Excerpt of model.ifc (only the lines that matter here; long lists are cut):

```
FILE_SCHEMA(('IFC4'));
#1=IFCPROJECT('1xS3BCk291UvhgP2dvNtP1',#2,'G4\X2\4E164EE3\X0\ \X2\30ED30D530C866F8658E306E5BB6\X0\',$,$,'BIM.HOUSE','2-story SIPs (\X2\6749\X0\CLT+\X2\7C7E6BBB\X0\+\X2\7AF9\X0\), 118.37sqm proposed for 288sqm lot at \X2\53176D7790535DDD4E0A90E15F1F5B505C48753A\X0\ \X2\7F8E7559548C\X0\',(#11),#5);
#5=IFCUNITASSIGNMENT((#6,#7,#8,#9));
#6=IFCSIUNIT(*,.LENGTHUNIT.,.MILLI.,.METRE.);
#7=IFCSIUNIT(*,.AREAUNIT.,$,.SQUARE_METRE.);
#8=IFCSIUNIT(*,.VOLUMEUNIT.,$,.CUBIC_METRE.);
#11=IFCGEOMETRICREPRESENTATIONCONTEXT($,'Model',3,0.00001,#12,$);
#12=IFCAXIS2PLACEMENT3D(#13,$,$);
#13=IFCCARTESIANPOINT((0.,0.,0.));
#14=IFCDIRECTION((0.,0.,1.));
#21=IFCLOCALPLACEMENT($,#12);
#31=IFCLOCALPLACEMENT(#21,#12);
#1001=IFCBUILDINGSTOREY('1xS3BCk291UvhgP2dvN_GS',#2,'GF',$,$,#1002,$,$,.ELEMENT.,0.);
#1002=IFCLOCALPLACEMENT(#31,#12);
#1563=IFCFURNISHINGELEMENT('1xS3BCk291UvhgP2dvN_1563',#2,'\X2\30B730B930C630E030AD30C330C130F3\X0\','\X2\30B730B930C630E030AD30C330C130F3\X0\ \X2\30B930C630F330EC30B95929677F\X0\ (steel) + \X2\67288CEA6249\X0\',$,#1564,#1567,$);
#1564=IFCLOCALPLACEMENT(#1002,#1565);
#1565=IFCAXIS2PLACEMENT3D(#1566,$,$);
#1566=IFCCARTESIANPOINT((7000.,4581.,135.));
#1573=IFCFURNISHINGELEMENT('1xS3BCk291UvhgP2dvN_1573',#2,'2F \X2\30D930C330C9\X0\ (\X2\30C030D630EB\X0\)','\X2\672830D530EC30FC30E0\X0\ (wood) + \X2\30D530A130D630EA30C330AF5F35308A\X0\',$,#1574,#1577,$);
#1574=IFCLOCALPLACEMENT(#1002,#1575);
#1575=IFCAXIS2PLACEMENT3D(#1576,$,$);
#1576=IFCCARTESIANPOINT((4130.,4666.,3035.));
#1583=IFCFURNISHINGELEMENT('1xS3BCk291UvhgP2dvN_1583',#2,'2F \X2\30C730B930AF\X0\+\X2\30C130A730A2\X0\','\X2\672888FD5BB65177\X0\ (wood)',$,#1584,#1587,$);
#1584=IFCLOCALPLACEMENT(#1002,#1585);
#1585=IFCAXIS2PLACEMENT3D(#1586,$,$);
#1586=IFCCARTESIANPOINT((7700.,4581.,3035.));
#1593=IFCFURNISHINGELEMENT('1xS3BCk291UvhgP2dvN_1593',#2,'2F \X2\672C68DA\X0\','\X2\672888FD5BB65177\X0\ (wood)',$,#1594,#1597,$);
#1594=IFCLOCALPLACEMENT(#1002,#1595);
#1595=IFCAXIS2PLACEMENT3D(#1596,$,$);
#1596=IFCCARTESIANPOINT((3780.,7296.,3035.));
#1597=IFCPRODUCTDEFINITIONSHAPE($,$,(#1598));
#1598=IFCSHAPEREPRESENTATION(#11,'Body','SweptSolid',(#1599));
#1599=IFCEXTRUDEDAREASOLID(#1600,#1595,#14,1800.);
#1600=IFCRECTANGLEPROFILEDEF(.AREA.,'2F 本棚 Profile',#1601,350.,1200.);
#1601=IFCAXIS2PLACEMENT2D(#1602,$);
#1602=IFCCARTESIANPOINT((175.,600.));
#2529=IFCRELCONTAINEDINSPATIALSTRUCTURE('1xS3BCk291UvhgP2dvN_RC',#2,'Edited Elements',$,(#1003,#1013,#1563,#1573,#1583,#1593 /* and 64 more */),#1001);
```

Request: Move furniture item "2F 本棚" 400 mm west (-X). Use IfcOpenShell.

```python
import ifcopenshell
import ifcopenshell.api.geometry
import ifcopenshell.util.placement
import ifcopenshell.util.unit

model = ifcopenshell.open("model.ifc")
unit_scale = ifcopenshell.util.unit.calculate_unit_scale(model)

item = model.by_guid("1xS3BCk291UvhgP2dvN_1593")
matrix = ifcopenshell.util.placement.get_local_placement(item.ObjectPlacement)
matrix[0, 3] -= 0.4 / unit_scale
ifcopenshell.api.geometry.edit_object_placement(model, product=item, matrix=matrix, is_si=False)

print(ifcopenshell.util.placement.get_local_placement(item.ObjectPlacement).round(3) + 0.0)

model.write("model_rev.ifc")
```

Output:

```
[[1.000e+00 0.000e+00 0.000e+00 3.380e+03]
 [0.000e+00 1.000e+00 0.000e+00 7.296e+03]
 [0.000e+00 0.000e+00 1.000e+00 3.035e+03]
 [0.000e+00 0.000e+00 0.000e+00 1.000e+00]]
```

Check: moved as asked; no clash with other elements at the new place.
